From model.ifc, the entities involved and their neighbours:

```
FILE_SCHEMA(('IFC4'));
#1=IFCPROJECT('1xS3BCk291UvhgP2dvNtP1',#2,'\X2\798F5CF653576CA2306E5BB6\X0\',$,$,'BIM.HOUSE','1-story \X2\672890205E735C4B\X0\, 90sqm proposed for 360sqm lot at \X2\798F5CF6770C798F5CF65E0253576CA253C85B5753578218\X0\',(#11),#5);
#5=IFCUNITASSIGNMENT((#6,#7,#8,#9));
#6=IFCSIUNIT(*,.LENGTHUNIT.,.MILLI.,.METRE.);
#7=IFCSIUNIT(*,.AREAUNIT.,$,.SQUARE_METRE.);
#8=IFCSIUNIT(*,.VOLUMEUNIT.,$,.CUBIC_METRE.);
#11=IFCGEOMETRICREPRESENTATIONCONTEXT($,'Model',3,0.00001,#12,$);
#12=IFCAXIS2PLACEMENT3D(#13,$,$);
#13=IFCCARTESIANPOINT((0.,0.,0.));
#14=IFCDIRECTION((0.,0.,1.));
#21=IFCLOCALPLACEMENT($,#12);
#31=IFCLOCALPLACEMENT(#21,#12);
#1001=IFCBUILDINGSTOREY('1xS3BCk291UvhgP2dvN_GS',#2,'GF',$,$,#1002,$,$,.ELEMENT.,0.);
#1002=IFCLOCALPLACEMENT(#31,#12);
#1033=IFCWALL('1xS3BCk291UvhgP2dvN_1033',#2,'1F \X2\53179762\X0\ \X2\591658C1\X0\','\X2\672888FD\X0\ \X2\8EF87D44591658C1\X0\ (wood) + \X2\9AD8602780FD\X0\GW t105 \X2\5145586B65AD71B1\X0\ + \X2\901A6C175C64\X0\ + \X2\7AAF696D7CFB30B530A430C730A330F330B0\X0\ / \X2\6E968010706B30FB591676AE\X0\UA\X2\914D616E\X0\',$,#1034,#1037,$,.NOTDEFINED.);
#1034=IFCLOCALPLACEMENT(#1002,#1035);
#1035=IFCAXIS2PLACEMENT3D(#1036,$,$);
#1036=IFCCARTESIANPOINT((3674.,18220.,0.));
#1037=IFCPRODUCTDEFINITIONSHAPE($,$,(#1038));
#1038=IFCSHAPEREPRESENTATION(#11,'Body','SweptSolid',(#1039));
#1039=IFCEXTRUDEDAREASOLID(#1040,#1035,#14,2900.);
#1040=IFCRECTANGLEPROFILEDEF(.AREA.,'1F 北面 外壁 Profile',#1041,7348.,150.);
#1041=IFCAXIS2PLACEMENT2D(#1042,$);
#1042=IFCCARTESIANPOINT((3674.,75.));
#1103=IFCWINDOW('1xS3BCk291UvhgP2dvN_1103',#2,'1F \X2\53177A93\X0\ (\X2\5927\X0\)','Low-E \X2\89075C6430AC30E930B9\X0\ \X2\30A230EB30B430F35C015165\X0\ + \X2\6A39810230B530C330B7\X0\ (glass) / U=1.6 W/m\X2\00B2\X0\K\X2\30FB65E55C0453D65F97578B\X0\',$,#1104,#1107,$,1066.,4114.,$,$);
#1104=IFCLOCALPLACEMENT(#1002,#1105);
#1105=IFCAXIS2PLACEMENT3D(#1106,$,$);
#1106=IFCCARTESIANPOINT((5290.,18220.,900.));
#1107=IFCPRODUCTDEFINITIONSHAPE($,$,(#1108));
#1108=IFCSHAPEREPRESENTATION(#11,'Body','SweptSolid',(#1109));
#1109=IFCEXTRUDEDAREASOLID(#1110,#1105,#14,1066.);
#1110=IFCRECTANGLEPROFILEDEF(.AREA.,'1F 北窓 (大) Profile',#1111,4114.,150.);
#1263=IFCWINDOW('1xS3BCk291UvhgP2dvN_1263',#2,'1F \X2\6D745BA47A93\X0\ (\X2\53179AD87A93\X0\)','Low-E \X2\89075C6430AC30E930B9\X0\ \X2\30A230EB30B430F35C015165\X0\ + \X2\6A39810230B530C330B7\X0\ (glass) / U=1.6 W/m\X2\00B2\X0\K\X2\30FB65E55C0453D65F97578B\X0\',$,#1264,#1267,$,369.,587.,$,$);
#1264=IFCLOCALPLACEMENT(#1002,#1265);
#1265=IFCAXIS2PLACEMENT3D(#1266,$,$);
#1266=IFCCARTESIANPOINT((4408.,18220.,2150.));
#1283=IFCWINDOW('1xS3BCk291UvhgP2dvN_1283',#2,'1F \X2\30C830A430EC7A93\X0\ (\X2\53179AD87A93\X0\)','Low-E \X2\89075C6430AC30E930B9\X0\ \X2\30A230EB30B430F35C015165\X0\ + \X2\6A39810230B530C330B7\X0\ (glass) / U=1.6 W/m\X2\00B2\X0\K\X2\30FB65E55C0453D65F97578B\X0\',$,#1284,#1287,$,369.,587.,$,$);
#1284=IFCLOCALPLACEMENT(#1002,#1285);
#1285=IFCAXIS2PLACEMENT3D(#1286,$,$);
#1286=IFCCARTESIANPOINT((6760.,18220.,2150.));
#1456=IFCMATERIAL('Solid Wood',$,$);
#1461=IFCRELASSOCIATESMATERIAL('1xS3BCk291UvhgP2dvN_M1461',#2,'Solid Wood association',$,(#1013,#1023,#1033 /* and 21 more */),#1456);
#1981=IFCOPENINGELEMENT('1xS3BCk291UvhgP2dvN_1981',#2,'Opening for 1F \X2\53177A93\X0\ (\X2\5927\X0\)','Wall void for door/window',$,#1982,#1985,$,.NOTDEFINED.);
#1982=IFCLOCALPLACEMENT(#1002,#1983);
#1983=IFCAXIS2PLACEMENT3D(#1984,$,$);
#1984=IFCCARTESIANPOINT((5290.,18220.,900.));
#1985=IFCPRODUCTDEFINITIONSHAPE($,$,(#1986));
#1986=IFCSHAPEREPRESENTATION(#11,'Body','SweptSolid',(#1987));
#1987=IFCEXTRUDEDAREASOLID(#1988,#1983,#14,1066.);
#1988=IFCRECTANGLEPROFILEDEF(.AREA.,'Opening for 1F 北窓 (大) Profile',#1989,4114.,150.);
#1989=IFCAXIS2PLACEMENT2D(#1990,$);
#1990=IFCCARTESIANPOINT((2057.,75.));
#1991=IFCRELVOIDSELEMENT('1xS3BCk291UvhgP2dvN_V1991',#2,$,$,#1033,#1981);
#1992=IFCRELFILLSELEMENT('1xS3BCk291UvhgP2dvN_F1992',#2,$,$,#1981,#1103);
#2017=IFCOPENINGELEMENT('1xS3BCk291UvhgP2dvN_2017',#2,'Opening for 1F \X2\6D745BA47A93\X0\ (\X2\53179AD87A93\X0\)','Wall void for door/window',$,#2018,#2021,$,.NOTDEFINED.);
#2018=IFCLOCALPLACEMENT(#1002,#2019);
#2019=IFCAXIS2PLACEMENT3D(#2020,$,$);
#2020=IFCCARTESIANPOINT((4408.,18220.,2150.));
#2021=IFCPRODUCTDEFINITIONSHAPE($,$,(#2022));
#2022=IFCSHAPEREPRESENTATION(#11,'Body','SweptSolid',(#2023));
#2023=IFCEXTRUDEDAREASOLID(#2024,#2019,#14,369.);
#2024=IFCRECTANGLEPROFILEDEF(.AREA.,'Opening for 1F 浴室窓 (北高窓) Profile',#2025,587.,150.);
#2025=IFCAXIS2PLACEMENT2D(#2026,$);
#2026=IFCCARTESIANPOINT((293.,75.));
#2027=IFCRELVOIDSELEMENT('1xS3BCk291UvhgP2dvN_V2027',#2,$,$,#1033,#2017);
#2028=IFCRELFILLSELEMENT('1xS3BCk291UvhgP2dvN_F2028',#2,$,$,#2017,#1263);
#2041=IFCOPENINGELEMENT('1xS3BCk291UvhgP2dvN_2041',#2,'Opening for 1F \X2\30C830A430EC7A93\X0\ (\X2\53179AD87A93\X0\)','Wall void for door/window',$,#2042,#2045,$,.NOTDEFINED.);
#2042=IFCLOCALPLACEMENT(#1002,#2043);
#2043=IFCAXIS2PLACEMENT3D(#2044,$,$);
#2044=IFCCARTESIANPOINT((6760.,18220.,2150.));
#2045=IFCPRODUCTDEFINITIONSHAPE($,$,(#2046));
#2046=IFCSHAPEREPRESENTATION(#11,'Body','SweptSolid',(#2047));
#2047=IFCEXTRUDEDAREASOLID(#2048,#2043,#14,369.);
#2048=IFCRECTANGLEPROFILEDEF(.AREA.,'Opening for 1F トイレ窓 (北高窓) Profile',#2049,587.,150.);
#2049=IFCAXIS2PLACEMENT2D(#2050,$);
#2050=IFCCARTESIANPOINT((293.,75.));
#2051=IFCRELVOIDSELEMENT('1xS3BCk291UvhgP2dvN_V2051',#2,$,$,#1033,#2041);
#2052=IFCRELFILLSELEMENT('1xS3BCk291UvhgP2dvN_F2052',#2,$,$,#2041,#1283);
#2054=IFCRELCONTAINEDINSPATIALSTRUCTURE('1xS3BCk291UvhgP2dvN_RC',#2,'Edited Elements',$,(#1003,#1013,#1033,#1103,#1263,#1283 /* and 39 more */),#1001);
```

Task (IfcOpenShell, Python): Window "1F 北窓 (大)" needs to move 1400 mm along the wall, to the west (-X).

```python
import ifcopenshell
import ifcopenshell.api.geometry
import ifcopenshell.util.placement
import ifcopenshell.util.unit

model = ifcopenshell.open("model.ifc")
unit_scale = ifcopenshell.util.unit.calculate_unit_scale(model)

window = model.by_id(1103)
opening = window.FillsVoids[0].RelatingOpeningElement
wall = opening.VoidsElements[0].RelatingBuildingElement

wall_matrix = ifcopenshell.util.placement.get_local_placement(wall.ObjectPlacement)
shift = wall_matrix[:3, 0] * -1.4 / unit_scale
before = ifcopenshell.util.placement.get_local_placement(window.ObjectPlacement)[:3, 3].copy()

# The window is not placed relative to its opening, so move both.
for product in (opening, window):
    matrix = ifcopenshell.util.placement.get_local_placement(product.ObjectPlacement)
    matrix[:3, 3] += shift
    ifcopenshell.api.geometry.edit_object_placement(model, product=product, matrix=matrix, is_si=False)

after = ifcopenshell.util.placement.get_local_placement(window.ObjectPlacement)[:3, 3]
print("window moved by", (after - before).round(3) + 0.0)

model.write("model_edited.ifc")
```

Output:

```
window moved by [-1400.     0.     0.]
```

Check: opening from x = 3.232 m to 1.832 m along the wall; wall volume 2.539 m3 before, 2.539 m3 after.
